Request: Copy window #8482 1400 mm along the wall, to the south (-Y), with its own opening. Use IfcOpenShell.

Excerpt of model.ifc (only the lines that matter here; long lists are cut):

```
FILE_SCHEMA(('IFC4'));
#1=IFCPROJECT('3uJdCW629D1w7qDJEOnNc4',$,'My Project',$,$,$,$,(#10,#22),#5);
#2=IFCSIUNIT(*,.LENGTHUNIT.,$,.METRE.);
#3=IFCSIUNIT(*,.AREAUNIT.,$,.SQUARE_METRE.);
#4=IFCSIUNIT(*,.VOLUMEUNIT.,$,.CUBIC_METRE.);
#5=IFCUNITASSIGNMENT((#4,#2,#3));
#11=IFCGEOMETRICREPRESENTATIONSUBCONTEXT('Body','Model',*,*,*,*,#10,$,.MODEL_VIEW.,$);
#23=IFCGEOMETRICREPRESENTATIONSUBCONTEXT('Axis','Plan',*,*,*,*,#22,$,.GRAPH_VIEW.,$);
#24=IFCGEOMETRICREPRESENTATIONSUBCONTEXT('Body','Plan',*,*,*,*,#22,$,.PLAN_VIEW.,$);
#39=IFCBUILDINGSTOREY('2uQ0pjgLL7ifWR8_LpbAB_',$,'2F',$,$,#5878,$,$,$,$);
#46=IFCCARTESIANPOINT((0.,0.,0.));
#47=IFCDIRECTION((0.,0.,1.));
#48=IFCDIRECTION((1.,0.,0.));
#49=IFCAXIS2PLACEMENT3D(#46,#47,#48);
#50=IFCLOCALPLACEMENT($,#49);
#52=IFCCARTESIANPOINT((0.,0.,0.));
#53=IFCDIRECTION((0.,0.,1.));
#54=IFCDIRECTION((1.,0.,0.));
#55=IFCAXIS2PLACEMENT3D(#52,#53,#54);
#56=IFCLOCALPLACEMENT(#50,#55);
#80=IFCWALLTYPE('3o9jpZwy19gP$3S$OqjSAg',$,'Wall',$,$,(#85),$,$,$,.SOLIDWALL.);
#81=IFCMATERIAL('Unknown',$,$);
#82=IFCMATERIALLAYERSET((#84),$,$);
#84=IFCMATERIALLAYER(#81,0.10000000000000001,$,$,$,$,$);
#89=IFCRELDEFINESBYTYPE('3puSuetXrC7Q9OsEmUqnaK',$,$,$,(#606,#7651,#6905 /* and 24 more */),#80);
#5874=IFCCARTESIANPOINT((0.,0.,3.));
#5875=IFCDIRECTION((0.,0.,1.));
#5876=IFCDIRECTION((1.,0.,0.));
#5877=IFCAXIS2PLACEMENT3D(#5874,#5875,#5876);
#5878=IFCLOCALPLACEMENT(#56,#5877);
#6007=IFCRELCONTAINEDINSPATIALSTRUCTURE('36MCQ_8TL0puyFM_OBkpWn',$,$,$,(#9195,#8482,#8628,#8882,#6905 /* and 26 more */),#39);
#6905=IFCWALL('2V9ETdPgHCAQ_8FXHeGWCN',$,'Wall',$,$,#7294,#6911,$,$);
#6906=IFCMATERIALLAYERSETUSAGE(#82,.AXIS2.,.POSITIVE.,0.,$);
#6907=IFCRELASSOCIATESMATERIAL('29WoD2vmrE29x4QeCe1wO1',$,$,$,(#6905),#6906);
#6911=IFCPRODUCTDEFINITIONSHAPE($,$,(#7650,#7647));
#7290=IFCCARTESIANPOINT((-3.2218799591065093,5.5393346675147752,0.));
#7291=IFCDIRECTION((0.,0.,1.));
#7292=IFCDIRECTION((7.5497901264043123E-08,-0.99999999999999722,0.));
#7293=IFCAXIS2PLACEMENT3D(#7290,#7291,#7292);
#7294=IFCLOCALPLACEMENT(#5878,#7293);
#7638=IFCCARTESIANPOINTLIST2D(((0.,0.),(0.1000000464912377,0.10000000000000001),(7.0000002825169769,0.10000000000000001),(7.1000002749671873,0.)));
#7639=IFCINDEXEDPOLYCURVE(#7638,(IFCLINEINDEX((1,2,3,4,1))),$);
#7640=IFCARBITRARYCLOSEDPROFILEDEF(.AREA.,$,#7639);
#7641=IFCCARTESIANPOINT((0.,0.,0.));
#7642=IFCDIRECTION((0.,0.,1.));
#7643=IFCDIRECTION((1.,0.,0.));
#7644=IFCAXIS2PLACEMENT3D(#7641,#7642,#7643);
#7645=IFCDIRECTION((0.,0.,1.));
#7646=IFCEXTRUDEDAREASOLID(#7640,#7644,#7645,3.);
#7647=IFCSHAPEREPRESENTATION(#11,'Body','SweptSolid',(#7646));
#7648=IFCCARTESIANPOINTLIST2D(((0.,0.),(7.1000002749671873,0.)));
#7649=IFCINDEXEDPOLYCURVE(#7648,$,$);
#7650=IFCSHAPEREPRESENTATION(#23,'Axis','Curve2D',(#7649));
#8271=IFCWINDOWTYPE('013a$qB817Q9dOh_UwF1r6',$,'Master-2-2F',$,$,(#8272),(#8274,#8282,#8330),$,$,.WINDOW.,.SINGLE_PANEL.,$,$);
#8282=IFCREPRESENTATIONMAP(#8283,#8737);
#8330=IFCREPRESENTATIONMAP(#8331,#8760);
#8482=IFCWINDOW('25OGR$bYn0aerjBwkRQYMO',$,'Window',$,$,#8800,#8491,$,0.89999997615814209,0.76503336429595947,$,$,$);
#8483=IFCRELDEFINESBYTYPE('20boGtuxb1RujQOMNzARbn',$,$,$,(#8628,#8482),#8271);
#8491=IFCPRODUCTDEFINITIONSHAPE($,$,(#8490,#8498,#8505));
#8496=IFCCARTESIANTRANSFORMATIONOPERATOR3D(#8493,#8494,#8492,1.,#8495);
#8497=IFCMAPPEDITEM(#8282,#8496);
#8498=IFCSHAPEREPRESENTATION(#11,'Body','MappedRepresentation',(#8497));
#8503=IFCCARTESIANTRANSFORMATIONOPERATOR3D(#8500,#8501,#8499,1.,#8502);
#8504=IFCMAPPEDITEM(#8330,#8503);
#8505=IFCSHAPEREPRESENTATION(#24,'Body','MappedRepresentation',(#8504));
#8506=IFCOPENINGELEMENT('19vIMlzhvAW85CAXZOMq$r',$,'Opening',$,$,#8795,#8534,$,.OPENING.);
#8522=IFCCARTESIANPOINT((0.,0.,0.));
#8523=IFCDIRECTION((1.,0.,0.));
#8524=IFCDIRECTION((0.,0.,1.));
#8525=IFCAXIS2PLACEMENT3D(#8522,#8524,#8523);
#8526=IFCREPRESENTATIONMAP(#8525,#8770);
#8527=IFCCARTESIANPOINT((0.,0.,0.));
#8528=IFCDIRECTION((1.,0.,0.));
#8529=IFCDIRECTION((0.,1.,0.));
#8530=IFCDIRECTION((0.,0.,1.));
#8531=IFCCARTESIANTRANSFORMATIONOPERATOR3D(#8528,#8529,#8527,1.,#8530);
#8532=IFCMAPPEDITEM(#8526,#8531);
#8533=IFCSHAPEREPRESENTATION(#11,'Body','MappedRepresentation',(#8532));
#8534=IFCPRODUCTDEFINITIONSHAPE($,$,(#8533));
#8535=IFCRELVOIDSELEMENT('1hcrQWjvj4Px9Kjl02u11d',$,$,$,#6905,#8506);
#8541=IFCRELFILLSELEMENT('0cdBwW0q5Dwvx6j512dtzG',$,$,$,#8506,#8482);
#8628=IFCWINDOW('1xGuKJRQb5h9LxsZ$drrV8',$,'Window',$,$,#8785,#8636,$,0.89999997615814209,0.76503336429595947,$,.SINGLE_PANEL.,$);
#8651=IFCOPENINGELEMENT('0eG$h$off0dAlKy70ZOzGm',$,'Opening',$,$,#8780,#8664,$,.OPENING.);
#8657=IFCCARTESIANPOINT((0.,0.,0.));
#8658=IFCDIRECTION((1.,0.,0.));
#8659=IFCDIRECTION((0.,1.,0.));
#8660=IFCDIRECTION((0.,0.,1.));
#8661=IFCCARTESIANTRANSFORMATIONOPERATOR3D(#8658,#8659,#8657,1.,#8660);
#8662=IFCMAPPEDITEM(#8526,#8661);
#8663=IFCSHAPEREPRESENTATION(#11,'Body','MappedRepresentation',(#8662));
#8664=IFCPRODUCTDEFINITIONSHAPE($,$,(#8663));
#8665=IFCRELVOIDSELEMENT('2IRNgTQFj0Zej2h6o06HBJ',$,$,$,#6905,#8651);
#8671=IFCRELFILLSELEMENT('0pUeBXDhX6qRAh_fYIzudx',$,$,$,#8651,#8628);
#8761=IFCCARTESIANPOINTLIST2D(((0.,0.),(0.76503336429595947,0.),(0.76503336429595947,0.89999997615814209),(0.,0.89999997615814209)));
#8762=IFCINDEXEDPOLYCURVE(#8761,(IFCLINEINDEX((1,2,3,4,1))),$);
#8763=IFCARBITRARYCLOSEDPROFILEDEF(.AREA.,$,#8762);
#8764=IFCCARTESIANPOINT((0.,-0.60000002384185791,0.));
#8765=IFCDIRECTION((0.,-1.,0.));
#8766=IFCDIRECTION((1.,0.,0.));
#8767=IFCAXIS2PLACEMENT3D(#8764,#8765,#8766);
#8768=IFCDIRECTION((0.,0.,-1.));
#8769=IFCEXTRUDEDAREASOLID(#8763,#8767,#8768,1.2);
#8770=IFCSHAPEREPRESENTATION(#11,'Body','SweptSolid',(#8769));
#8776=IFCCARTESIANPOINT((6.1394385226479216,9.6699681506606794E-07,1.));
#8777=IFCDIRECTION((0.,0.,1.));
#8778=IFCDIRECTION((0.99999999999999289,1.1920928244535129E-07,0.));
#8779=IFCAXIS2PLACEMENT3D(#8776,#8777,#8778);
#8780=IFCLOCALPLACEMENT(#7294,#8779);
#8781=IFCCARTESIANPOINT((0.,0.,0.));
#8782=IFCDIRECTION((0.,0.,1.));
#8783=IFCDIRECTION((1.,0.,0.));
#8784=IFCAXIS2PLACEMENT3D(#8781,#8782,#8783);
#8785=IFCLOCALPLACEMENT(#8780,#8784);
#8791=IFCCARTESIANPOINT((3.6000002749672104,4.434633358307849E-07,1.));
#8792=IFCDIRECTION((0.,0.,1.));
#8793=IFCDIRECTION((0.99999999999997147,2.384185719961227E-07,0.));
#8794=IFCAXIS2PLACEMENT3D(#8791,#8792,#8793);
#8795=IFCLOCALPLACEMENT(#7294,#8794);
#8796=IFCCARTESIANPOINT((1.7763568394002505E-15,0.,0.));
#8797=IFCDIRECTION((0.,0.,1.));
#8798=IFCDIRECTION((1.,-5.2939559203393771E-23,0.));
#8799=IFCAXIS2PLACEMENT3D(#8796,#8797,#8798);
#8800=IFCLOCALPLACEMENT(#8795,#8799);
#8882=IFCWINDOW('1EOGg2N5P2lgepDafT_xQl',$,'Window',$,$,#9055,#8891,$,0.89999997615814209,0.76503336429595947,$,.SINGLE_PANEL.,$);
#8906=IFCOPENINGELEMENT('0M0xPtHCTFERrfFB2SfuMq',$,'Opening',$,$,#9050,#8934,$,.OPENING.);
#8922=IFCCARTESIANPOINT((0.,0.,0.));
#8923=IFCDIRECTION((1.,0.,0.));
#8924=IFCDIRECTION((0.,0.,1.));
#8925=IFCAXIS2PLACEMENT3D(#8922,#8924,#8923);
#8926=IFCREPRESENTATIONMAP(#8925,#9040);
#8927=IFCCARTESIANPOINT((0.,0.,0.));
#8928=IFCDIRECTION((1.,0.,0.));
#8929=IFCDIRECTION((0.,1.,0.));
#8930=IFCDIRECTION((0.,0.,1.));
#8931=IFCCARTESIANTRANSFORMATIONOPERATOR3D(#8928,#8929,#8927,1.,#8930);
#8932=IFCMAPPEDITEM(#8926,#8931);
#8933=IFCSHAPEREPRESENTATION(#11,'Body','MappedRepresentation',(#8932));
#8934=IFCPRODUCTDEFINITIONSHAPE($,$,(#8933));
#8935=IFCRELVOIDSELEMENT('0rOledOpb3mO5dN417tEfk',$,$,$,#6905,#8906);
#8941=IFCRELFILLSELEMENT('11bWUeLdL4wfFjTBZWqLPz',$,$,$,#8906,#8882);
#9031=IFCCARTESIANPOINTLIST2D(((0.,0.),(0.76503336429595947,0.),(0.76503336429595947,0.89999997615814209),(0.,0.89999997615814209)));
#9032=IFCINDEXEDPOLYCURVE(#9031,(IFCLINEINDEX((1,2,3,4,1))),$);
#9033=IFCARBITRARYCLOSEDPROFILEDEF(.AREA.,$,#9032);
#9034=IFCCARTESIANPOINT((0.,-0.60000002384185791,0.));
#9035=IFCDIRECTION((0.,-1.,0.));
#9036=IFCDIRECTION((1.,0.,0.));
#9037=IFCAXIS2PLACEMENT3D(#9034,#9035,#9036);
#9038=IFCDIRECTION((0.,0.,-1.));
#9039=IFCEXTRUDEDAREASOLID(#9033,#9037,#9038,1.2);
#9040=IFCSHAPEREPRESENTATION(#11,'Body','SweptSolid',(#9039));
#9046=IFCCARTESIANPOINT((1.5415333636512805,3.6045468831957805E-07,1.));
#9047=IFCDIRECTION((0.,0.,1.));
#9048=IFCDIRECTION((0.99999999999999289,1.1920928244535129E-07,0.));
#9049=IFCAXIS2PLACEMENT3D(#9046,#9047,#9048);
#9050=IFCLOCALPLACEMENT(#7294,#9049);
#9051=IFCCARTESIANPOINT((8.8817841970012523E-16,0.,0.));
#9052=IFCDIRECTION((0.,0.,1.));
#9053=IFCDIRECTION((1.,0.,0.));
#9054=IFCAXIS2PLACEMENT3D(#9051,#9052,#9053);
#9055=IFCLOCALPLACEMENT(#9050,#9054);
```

```python
import ifcopenshell
import ifcopenshell.api.feature
import ifcopenshell.api.geometry
import ifcopenshell.api.root
import ifcopenshell.geom
import ifcopenshell.util.element
import ifcopenshell.util.placement
import ifcopenshell.util.shape

model = ifcopenshell.open("model.ifc")
settings = ifcopenshell.geom.settings()


def volume(element):
    """Net volume in cubic metres, openings subtracted."""
    shape = ifcopenshell.geom.create_shape(settings, element)
    return ifcopenshell.util.shape.get_volume(shape.geometry)


window = model.by_guid("25OGR$bYn0aerjBwkRQYMO")
opening = window.FillsVoids[0].RelatingOpeningElement
wall = opening.VoidsElements[0].RelatingBuildingElement
before = volume(wall)
shift = ifcopenshell.util.placement.get_local_placement(wall.ObjectPlacement)[:3, 0] * 1.4

# copy_class copies the void relationship, type, container and properties, but no geometry.
new_opening = ifcopenshell.api.root.copy_class(model, product=opening)
new_opening.Representation = ifcopenshell.util.element.copy_deep(
    model, opening.Representation, exclude=["IfcGeometricRepresentationContext", "IfcRepresentationMap"]
)
new_window = ifcopenshell.api.root.copy_class(model, product=window)
new_window.Representation = ifcopenshell.util.element.copy_deep(
    model, window.Representation, exclude=["IfcGeometricRepresentationContext", "IfcRepresentationMap"]
)
ifcopenshell.api.feature.add_filling(model, opening=new_opening, element=new_window)

for old, new in ((opening, new_opening), (window, new_window)):
    matrix = ifcopenshell.util.placement.get_local_placement(old.ObjectPlacement)
    matrix[:3, 3] += shift
    ifcopenshell.api.geometry.edit_object_placement(model, product=new, matrix=matrix, is_si=False)

after = volume(wall)

print(f"wall volume {before:.3f} -> {after:.3f} m3")

model.write("model_v2.ifc")
```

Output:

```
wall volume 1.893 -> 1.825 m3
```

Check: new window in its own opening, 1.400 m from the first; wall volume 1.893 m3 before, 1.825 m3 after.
